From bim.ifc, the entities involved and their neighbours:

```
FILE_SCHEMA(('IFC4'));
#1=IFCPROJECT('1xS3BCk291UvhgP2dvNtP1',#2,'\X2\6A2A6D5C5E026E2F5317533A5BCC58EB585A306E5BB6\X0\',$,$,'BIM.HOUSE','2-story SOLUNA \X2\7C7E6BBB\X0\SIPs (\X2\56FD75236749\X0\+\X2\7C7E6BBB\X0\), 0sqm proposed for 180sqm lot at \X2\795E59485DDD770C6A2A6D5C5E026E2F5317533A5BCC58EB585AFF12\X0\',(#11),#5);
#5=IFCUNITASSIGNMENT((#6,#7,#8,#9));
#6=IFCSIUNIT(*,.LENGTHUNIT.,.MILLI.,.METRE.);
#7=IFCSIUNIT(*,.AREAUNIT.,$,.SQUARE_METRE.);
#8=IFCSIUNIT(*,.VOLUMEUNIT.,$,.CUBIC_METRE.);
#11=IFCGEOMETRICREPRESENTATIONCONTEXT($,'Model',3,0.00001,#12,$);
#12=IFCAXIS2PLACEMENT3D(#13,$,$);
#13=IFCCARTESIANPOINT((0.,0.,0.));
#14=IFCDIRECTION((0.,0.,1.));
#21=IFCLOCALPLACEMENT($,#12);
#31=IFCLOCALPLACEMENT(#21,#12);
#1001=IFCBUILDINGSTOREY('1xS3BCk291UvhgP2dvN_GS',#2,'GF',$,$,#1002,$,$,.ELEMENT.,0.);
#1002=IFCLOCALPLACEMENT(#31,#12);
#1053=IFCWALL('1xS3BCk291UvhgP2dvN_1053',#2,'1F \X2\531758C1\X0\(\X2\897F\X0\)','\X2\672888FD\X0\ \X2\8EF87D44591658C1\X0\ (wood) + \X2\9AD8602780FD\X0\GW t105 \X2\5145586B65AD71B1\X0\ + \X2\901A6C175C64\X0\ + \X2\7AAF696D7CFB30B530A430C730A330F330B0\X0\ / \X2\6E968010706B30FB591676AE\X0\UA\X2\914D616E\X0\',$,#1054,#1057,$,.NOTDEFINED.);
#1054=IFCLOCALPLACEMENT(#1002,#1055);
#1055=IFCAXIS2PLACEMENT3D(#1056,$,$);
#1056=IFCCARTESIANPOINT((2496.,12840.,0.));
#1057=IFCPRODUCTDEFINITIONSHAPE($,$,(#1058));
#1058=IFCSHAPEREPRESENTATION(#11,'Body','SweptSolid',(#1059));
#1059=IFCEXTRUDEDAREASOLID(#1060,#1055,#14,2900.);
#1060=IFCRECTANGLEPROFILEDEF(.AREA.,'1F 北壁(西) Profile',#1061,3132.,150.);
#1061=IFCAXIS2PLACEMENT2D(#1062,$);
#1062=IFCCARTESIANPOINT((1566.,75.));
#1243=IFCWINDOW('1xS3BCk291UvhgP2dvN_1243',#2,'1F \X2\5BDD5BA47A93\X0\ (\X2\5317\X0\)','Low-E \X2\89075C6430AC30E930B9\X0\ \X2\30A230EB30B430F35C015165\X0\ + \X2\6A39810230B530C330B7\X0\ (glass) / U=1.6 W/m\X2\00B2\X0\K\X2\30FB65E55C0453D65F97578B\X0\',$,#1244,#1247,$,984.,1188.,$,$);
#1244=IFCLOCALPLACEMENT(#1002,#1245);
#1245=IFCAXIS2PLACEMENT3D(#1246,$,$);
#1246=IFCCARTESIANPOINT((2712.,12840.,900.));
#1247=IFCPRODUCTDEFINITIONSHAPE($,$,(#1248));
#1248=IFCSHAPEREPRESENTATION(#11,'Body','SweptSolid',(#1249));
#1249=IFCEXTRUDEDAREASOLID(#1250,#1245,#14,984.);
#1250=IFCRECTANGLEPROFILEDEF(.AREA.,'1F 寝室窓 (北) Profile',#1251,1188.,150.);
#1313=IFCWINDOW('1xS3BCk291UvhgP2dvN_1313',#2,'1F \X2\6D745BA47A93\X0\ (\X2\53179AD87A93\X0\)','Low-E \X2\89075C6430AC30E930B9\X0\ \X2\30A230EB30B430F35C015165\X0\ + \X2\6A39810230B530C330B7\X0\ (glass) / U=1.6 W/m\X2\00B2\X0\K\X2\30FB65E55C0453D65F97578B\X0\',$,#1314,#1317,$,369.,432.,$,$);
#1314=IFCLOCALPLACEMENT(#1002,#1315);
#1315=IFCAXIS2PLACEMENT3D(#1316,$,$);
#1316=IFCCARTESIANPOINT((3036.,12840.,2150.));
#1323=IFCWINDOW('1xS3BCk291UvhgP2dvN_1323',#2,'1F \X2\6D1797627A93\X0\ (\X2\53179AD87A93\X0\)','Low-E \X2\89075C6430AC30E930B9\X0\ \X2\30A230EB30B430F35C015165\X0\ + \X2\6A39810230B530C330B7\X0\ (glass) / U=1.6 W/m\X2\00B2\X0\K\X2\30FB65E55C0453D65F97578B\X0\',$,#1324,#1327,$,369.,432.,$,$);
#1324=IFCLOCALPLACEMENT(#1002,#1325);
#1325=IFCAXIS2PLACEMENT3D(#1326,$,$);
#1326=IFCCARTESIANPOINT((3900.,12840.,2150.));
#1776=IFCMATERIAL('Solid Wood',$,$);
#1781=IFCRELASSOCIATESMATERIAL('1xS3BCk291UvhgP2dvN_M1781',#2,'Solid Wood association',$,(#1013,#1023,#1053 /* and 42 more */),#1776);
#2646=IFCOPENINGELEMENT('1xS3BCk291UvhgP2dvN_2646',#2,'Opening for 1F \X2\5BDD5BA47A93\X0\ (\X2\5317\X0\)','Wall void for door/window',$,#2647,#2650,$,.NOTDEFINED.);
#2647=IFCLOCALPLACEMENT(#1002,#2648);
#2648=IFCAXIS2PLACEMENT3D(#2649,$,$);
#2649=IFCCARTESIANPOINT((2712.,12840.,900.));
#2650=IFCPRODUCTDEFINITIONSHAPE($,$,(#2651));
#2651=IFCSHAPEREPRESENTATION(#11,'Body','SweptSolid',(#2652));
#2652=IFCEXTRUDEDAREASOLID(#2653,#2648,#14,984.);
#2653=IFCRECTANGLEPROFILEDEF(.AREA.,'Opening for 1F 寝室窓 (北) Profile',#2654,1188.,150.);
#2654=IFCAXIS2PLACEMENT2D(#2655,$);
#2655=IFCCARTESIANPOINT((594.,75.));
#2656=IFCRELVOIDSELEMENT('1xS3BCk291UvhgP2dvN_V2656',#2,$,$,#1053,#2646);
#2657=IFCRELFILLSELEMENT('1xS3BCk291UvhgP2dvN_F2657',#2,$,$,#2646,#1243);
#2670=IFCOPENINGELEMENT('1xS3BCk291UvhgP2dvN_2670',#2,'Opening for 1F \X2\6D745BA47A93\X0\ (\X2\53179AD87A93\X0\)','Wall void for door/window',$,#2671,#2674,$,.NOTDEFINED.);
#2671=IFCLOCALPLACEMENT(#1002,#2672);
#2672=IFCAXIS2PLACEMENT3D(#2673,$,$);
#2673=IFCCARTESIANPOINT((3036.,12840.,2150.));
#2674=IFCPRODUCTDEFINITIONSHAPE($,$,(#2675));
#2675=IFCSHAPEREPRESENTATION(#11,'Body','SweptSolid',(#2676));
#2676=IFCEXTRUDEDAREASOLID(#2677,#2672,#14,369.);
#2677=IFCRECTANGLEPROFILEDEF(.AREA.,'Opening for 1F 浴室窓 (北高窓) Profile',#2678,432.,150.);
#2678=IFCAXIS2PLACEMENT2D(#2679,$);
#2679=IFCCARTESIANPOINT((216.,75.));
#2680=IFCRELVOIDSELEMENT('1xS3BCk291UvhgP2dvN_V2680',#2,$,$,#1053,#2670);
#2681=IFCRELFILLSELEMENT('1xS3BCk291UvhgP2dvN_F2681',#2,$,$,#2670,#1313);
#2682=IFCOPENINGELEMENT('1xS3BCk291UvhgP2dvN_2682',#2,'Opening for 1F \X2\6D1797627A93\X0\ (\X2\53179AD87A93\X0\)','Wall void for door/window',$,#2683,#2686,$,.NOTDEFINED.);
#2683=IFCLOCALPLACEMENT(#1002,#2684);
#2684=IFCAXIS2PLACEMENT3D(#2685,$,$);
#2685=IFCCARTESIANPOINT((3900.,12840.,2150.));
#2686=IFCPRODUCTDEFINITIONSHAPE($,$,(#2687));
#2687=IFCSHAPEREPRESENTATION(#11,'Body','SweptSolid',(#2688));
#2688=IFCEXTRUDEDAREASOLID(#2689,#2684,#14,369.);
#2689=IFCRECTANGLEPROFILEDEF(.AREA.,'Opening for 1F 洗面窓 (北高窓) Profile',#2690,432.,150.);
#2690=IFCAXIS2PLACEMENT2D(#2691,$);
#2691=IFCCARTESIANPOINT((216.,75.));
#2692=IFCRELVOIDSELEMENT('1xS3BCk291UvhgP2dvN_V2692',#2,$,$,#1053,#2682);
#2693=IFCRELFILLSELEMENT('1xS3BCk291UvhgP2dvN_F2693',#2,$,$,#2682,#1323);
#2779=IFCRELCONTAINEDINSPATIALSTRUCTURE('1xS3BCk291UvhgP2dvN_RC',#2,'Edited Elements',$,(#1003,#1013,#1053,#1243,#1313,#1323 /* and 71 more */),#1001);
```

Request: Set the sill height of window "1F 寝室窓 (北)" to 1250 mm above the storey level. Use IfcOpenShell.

```python
import numpy as np
import ifcopenshell
import ifcopenshell.api.geometry
import ifcopenshell.geom
import ifcopenshell.util.element
import ifcopenshell.util.placement
import ifcopenshell.util.shape
import ifcopenshell.util.unit

model = ifcopenshell.open("bim.ifc")
unit_scale = ifcopenshell.util.unit.calculate_unit_scale(model)

window = model.by_guid("1xS3BCk291UvhgP2dvN_1243")
opening = window.FillsVoids[0].RelatingOpeningElement
storey = ifcopenshell.util.element.get_container(window, ifc_class="IfcBuildingStorey")
level = ifcopenshell.util.placement.get_local_placement(storey.ObjectPlacement)[2, 3]

# The opening's origin need not be at the sill, so measure its lowest point.
shape = ifcopenshell.geom.create_shape(ifcopenshell.geom.settings(), opening)
bottom = ifcopenshell.util.shape.get_shape_bottom_elevation(shape, shape.geometry) / unit_scale
dz = level + 1.25 / unit_scale - bottom

shift = np.array([0.0, 0.0, dz])
# The window is not placed relative to its opening, so move both.
for product in (opening, window):
    matrix = ifcopenshell.util.placement.get_local_placement(product.ObjectPlacement)
    matrix[:3, 3] += shift
    ifcopenshell.api.geometry.edit_object_placement(model, product=product, matrix=matrix, is_si=False)

print(f"moved by {dz * unit_scale:+.3f} m")

model.write("bim_rev.ifc")
```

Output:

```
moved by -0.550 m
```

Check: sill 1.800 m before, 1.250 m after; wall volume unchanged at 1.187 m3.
